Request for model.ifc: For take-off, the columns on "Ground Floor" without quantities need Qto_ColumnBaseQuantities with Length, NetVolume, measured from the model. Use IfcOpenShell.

First a look at what the model holds.

```python
import ifcopenshell
import ifcopenshell.util.element
import ifcopenshell.util.unit

model = ifcopenshell.open("model.ifc")
print(model.schema)
for unit_type in ("LENGTHUNIT", "AREAUNIT", "VOLUMEUNIT"):
    print(unit_type, ifcopenshell.util.unit.calculate_unit_scale(model, unit_type))
storey = next(s for s in model.by_type("IfcBuildingStorey") if s.Name == "Ground Floor")
columns = [e for e in ifcopenshell.util.element.get_decomposition(storey) if e.is_a("IfcColumn")]
for e in sorted(columns, key=lambda e: e.id()):
    print(e.id(), e.is_a(), e.Name, list(ifcopenshell.util.element.get_psets(e, qtos_only=True)), sep=" | ")
```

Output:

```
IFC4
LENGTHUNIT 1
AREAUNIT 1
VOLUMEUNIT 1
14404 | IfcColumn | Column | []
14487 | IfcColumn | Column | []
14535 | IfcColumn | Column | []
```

```python
import ifcopenshell
import ifcopenshell.api.pset
import ifcopenshell.geom
import ifcopenshell.util.element
import ifcopenshell.util.shape
import ifcopenshell.util.unit

model = ifcopenshell.open("model.ifc")
unit_scale = ifcopenshell.util.unit.calculate_unit_scale(model)
volume_scale = ifcopenshell.util.unit.calculate_unit_scale(model, "VOLUMEUNIT")
settings = ifcopenshell.geom.settings()

storey = next(s for s in model.by_type("IfcBuildingStorey") if s.Name == "Ground Floor")
columns = [e for e in ifcopenshell.util.element.get_decomposition(storey) if e.is_a("IfcColumn")]

for e in sorted(columns, key=lambda e: e.id()):
    if ifcopenshell.util.element.get_psets(e, qtos_only=True, should_inherit=False):
        continue
    # Geometry comes back in metres, in the element's own axes.
    shape = ifcopenshell.geom.create_shape(settings, e)
    values = {
        "Length": ifcopenshell.util.shape.get_z(shape.geometry) / unit_scale,
        "NetVolume": ifcopenshell.util.shape.get_volume(shape.geometry) / volume_scale,
    }
    qto = ifcopenshell.api.pset.add_qto(model, product=e, name="Qto_ColumnBaseQuantities")
    ifcopenshell.api.pset.edit_qto(model, qto=qto, properties=values)
    print(e.id(), {k: round(v, 3) for k, v in values.items()})

model.write("model_updated.ifc")
```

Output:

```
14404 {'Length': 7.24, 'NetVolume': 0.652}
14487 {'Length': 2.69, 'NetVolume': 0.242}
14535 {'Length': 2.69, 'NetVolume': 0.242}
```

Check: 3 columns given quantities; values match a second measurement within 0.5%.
